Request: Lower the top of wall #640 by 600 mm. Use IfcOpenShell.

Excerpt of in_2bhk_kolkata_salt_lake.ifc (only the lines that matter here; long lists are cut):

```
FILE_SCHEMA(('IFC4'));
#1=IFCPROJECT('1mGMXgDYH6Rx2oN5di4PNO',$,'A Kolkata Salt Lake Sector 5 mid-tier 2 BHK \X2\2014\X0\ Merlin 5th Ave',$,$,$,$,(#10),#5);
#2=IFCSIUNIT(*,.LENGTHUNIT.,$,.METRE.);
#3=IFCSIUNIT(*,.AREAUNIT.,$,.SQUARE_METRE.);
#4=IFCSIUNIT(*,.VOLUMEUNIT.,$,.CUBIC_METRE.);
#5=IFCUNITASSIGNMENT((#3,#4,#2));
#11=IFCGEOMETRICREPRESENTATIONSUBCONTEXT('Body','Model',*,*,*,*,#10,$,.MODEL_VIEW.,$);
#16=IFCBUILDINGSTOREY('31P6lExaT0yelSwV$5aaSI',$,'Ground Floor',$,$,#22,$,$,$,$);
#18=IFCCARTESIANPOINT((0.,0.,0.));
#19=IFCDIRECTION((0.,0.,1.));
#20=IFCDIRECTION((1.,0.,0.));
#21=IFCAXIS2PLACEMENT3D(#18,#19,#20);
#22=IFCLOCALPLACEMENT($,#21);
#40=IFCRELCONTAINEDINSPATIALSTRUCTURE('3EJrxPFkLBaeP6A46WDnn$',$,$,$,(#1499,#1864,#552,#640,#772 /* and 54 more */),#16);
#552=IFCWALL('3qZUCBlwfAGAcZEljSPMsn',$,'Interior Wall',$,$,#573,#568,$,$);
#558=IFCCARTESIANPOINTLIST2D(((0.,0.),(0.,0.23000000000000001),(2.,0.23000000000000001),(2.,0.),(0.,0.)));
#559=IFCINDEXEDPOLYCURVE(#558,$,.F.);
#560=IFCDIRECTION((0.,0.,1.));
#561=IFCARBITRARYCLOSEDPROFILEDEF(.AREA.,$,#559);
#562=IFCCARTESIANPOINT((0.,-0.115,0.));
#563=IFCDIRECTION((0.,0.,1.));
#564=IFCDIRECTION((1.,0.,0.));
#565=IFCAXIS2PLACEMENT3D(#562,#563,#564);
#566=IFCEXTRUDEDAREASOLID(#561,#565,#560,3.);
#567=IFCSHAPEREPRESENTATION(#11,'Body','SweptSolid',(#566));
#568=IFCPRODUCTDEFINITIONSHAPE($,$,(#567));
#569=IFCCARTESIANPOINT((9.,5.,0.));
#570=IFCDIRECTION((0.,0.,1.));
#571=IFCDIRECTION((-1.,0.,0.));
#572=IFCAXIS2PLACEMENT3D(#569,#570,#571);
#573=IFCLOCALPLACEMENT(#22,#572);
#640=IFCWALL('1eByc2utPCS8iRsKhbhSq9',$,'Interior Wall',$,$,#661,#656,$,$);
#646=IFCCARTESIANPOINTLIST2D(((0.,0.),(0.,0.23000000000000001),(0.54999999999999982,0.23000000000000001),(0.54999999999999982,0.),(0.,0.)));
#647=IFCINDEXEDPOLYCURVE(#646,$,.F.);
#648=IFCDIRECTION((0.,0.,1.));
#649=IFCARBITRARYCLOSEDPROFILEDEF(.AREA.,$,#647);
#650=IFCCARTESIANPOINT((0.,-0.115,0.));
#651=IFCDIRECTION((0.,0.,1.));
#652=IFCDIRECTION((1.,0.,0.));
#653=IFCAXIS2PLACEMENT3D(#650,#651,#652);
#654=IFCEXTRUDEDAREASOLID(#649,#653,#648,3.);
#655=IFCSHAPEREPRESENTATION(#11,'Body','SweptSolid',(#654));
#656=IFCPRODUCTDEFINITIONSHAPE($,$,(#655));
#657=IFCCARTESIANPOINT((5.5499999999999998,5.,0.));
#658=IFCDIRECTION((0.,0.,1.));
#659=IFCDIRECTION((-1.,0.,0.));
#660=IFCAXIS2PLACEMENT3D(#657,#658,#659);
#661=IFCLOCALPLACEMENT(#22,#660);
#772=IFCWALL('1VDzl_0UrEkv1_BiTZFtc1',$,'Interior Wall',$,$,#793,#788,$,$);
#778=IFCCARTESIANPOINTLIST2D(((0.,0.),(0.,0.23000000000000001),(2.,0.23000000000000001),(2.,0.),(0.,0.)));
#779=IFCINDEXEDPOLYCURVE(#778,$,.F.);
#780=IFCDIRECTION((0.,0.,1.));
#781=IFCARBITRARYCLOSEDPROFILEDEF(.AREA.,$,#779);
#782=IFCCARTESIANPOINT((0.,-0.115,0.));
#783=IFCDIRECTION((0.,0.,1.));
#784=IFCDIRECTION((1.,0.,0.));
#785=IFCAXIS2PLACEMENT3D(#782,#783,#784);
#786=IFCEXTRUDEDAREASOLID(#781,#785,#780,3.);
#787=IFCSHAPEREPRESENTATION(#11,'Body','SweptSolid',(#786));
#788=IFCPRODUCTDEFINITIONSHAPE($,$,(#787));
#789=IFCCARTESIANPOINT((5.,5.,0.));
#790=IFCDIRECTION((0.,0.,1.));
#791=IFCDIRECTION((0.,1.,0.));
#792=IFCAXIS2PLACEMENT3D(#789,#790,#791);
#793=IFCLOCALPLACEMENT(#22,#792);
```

```python
import ifcopenshell
import ifcopenshell.geom
import ifcopenshell.util.representation
import ifcopenshell.util.shape
import ifcopenshell.util.unit

model = ifcopenshell.open("in_2bhk_kolkata_salt_lake.ifc")
unit_scale = ifcopenshell.util.unit.calculate_unit_scale(model)
settings = ifcopenshell.geom.settings()


def volume(element):
    """Net volume in cubic metres, openings subtracted."""
    shape = ifcopenshell.geom.create_shape(settings, element)
    return ifcopenshell.util.shape.get_volume(shape.geometry)


wall = model.by_guid("1eByc2utPCS8iRsKhbhSq9")
before = volume(wall)

body = ifcopenshell.util.representation.get_representation(wall, "Model", "Body")
solid = body.Items[0]
old_height = solid.Depth
solid.Depth -= 0.6 / unit_scale
after = volume(wall)

print(f"height {old_height:g} -> {solid.Depth:g}, volume {before:.3f} -> {after:.3f} m3")

model.write("in_2bhk_kolkata_salt_lake_rev.ifc")
```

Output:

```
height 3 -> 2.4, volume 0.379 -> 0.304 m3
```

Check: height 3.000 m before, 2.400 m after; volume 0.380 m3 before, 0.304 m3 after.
